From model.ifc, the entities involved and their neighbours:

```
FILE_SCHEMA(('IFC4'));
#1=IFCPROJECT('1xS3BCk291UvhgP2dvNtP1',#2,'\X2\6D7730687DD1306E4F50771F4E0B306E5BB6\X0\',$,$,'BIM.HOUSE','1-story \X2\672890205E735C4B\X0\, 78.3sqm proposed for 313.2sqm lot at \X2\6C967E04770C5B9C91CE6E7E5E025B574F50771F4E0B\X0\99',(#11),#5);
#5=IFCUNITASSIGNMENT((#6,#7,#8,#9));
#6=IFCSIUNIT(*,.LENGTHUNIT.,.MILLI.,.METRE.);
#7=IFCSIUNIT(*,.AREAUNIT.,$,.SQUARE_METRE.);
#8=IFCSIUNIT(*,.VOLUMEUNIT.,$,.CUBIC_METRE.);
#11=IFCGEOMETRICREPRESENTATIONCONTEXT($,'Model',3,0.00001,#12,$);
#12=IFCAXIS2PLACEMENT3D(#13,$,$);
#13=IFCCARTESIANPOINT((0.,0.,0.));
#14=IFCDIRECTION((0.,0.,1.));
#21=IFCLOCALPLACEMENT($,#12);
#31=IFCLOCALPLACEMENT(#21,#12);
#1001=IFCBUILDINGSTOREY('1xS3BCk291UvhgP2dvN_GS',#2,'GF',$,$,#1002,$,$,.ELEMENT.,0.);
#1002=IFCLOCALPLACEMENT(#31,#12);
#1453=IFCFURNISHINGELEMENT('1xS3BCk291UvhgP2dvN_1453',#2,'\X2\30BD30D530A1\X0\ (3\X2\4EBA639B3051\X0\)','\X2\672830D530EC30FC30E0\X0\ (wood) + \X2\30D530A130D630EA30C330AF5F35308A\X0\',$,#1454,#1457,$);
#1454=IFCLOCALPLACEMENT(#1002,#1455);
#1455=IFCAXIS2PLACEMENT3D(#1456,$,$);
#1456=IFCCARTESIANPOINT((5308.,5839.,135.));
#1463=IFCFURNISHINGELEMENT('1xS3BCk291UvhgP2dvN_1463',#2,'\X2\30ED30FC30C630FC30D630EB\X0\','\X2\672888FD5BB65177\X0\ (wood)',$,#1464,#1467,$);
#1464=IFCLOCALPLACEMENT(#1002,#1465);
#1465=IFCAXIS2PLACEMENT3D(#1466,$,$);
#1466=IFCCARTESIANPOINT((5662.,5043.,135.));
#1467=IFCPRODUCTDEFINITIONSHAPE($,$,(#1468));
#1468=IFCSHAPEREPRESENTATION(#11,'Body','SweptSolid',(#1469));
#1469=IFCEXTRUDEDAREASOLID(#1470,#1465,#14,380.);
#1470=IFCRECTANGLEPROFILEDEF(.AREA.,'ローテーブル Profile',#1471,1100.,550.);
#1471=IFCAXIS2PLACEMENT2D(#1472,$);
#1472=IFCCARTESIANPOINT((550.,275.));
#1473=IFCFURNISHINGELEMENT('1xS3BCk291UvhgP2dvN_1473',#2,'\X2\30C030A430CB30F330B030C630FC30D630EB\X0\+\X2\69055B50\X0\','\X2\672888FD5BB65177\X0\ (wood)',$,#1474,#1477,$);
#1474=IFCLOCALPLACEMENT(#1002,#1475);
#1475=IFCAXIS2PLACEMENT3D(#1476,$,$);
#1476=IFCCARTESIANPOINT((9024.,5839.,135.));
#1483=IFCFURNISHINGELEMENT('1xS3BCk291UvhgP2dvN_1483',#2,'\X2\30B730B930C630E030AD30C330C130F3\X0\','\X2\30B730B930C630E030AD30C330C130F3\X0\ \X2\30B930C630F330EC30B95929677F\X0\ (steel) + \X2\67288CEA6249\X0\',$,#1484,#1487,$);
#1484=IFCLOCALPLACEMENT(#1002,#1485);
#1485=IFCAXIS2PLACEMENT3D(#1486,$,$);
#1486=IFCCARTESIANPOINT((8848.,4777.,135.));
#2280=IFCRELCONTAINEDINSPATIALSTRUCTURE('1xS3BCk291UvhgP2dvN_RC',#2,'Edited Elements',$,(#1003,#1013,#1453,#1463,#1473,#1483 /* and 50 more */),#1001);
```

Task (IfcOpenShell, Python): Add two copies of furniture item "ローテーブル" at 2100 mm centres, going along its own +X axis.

```python
import ifcopenshell
import ifcopenshell.api.geometry
import ifcopenshell.api.root
import ifcopenshell.util.element
import ifcopenshell.util.placement

model = ifcopenshell.open("model.ifc")


def reuse_history(source, copy):
    """copy_class also copies each property set's owner history, people and application; keep the originals."""
    for rel in copy.IsDefinedBy:
        if rel.is_a("IfcRelDefinesByProperties") and (history := rel.RelatingPropertyDefinition.OwnerHistory):
            rel.RelatingPropertyDefinition.OwnerHistory = source.OwnerHistory
            ifcopenshell.util.element.remove_deep2(model, history)


source = model.by_id(1463)
base = ifcopenshell.util.placement.get_local_placement(source.ObjectPlacement)
step = base[:3, 0] * 2100.0

for i in range(1, 3):
    copy = ifcopenshell.api.root.copy_class(model, product=source)
    copy.Representation = ifcopenshell.util.element.copy_deep(
        model, source.Representation, exclude=["IfcGeometricRepresentationContext", "IfcRepresentationMap"]
    )
    reuse_history(source, copy)
    matrix = base.copy()
    matrix[:3, 3] += i * step
    print("added at", matrix[:3, 3].round(3) + 0.0)
    ifcopenshell.api.geometry.edit_object_placement(model, product=copy, matrix=matrix, is_si=False)

model.write("model_v2.ifc")
```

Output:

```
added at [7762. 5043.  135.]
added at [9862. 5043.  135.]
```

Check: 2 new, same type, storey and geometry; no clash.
